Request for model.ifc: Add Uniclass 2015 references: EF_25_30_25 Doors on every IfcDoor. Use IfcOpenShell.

First a look at what the model holds.

```python
import ifcopenshell

model = ifcopenshell.open("model.ifc")
print(model.schema)
print("classifications:", [c.Name for c in model.by_type("IfcClassification")])
for ifc_class in ("IfcDoor", "IfcRoof", "IfcStair", "IfcWall", "IfcWindow"):
    print(ifc_class, len(model.by_type(ifc_class)))
```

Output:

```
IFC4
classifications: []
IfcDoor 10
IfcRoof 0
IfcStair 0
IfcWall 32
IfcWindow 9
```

```python
import ifcopenshell
import ifcopenshell.api.classification

model = ifcopenshell.open("model.ifc")

system = ifcopenshell.api.classification.add_classification(model, classification="Uniclass 2015")

codes = {
    "IfcDoor": ("EF_25_30_25", "Doors"),
}
for ifc_class, (code, name) in codes.items():
    products = model.by_type(ifc_class)
    ifcopenshell.api.classification.add_reference(
        model, products=products, classification=system, identification=code, name=name
    )
    print(code, len(products))

model.write("model_edited.ifc")
```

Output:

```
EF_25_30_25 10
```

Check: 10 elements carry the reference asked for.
